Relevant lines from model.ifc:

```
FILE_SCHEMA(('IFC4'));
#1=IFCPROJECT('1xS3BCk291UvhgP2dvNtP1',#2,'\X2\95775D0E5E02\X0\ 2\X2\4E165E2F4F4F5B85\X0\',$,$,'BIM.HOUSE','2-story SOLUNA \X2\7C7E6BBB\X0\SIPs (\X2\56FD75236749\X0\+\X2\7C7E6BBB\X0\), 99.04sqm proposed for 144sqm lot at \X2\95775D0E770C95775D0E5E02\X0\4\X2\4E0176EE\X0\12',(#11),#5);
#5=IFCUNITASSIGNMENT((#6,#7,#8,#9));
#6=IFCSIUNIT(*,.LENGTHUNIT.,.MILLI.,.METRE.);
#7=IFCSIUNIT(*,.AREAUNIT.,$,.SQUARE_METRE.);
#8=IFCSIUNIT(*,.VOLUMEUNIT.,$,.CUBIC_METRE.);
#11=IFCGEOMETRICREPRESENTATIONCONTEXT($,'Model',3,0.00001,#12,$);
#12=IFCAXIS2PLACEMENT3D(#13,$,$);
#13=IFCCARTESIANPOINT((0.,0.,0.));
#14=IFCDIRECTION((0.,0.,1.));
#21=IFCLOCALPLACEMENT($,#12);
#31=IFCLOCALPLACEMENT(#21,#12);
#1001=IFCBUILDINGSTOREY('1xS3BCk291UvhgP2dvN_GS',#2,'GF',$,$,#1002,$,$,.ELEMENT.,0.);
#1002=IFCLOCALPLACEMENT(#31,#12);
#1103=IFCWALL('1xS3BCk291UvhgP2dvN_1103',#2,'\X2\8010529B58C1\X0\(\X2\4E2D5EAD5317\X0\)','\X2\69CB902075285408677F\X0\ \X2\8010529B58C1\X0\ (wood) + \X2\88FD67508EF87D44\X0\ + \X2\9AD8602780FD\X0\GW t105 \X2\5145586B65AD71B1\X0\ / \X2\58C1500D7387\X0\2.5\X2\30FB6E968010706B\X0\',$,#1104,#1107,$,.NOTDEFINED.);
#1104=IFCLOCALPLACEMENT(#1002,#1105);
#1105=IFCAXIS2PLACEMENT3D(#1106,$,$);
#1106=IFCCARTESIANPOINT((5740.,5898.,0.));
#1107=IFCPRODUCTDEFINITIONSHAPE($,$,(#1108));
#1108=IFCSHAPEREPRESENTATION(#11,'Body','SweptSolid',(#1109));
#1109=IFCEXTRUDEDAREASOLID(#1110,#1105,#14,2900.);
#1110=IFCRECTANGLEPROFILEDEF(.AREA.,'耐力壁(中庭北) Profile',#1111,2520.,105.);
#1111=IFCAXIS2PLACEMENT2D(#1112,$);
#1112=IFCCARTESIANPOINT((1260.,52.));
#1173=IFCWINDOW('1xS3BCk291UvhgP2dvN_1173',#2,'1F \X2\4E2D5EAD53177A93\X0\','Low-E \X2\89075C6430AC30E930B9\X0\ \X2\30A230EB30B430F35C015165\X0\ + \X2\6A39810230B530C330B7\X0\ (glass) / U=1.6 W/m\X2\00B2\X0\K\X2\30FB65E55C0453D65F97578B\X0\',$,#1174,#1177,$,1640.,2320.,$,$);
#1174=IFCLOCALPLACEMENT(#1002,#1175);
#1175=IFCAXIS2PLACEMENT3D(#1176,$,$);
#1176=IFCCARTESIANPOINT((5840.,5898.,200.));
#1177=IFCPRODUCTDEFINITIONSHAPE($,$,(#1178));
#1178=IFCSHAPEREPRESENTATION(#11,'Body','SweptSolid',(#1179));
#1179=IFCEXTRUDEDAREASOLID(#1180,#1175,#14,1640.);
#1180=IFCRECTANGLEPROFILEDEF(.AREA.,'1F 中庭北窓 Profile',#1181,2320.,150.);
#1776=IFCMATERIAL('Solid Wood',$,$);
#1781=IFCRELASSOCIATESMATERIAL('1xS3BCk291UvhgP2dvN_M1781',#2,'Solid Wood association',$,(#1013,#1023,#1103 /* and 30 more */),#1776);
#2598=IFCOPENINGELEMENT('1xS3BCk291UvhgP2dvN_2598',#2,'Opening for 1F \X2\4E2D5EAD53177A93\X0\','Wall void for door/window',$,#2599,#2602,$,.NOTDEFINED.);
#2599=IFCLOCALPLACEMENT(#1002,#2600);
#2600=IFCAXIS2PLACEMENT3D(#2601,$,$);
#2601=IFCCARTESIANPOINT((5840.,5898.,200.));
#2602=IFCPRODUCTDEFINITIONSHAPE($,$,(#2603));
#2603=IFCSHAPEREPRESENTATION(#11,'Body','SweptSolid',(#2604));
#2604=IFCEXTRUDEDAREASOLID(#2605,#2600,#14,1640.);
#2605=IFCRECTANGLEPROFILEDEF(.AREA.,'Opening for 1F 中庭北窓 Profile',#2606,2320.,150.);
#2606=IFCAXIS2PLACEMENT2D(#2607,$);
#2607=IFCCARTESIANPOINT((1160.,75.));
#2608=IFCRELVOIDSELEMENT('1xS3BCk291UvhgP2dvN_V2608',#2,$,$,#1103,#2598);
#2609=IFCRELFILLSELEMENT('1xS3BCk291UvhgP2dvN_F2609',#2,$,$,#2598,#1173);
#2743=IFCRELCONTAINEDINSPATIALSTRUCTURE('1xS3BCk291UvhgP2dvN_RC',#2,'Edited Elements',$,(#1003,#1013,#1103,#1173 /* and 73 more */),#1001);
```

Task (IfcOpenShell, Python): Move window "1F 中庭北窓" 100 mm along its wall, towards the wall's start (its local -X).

```python
import ifcopenshell
import ifcopenshell.api.geometry
import ifcopenshell.util.placement
import ifcopenshell.util.unit

model = ifcopenshell.open("model.ifc")
unit_scale = ifcopenshell.util.unit.calculate_unit_scale(model)

window = model.by_id(1173)
opening = window.FillsVoids[0].RelatingOpeningElement
wall = opening.VoidsElements[0].RelatingBuildingElement

wall_matrix = ifcopenshell.util.placement.get_local_placement(wall.ObjectPlacement)
shift = wall_matrix[:3, 0] * -0.1 / unit_scale
before = ifcopenshell.util.placement.get_local_placement(window.ObjectPlacement)[:3, 3].copy()

# The window is not placed relative to its opening, so move both.
for product in (opening, window):
    matrix = ifcopenshell.util.placement.get_local_placement(product.ObjectPlacement)
    matrix[:3, 3] += shift
    ifcopenshell.api.geometry.edit_object_placement(model, product=product, matrix=matrix, is_si=False)

after = ifcopenshell.util.placement.get_local_placement(window.ObjectPlacement)[:3, 3]
print("window moved by", (after - before).round(3) + 0.0)

model.write("model_rev.ifc")
```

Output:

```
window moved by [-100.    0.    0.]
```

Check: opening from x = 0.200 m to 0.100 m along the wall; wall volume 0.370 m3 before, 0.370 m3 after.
